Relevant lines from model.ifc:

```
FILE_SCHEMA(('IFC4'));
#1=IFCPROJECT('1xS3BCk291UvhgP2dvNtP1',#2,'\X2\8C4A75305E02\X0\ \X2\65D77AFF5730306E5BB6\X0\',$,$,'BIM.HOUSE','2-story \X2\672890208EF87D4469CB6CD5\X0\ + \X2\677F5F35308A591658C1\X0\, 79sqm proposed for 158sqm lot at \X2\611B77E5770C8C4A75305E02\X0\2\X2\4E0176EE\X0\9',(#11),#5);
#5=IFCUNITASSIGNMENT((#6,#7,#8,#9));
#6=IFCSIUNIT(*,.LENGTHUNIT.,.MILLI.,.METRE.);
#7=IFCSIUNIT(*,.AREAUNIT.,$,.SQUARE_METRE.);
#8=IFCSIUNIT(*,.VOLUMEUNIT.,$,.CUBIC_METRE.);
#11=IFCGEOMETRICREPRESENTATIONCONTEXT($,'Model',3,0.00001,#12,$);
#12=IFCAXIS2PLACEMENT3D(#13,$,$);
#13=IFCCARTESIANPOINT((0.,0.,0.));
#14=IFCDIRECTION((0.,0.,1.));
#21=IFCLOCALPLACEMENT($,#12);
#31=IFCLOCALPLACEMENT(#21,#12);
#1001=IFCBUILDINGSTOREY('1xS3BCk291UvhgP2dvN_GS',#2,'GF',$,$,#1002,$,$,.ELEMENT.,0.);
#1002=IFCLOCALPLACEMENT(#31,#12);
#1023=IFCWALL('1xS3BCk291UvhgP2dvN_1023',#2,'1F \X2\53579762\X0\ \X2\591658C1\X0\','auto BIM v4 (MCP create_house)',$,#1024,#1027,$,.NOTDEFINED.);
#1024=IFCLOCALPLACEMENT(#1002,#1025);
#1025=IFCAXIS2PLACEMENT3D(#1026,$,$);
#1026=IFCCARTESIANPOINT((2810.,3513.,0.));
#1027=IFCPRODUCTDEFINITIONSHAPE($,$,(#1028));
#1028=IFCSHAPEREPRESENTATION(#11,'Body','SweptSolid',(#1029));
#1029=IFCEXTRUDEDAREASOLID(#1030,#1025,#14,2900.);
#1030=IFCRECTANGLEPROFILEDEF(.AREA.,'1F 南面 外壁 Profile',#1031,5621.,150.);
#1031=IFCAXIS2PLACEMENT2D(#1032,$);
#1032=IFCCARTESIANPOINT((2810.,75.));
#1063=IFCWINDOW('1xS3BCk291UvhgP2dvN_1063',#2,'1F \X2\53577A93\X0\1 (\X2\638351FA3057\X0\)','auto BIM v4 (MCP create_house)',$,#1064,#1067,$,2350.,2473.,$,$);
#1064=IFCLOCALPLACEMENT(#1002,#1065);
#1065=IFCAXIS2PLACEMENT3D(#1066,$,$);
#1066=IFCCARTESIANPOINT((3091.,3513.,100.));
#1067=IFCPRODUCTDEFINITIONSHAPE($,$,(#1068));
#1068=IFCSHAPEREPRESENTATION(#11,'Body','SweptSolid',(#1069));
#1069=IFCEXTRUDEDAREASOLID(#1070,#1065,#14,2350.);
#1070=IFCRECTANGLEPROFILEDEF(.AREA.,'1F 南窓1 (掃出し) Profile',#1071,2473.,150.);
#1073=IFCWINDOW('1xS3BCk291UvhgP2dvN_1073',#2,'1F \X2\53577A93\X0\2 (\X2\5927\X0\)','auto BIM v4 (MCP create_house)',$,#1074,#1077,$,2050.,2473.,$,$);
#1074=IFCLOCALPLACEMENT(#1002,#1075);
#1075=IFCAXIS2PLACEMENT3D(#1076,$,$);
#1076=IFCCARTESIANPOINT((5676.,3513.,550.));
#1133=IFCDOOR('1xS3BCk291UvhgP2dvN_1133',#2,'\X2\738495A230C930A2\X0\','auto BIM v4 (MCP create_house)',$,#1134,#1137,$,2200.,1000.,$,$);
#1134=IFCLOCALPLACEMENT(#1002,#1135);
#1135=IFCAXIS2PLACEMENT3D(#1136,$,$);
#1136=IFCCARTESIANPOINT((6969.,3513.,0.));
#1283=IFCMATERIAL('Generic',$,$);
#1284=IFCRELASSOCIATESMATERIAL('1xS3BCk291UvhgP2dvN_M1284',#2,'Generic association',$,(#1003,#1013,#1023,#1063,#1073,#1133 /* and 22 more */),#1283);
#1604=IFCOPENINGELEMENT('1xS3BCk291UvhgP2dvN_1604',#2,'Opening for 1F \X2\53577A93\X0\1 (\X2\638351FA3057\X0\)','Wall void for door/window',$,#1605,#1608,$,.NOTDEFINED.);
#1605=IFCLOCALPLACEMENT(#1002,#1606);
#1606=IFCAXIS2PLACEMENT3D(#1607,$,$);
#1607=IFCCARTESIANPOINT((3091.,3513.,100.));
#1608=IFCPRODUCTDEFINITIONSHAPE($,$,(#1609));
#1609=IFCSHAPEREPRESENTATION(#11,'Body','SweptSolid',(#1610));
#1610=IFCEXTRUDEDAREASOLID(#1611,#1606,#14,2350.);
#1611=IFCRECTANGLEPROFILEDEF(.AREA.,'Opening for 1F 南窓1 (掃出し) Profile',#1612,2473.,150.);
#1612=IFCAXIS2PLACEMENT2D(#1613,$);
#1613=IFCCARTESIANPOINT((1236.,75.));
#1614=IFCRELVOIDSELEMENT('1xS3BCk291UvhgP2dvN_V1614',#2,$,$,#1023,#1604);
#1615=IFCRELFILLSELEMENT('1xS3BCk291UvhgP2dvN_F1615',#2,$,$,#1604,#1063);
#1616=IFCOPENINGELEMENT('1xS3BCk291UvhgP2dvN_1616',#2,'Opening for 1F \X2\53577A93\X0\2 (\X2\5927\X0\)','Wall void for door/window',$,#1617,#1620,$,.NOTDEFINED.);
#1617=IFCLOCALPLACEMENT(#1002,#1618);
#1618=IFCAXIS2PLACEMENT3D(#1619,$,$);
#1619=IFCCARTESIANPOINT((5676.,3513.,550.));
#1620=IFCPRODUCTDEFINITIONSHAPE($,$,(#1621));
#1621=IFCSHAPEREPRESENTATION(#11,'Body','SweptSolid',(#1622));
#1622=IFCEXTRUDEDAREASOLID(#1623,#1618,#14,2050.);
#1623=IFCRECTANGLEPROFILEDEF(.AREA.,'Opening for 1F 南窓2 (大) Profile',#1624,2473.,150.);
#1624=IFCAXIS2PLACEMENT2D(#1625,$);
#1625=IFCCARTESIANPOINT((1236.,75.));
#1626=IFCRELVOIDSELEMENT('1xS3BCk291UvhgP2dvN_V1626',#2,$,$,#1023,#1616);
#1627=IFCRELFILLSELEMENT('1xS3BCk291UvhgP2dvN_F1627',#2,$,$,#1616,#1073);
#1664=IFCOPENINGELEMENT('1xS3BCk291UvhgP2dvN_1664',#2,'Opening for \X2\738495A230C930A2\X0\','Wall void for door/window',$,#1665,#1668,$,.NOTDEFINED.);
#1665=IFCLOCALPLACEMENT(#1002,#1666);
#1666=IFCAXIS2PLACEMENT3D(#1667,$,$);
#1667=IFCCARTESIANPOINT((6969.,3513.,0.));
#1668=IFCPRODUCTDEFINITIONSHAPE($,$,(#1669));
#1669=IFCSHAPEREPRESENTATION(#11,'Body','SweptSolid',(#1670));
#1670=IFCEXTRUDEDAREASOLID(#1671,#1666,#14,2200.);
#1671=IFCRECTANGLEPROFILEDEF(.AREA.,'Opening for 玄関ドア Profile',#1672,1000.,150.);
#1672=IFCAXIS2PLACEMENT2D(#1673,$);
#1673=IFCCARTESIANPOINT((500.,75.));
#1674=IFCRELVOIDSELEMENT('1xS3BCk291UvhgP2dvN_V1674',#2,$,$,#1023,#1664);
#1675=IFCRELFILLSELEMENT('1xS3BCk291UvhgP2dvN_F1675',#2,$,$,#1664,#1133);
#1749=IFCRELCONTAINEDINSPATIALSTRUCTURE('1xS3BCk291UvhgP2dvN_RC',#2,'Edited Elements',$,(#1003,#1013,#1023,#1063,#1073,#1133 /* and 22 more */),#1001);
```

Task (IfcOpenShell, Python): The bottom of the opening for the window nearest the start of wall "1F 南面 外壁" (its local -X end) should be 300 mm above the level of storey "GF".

```python
import numpy as np
import ifcopenshell
import ifcopenshell.api.geometry
import ifcopenshell.geom
import ifcopenshell.util.element
import ifcopenshell.util.placement
import ifcopenshell.util.shape
import ifcopenshell.util.unit

model = ifcopenshell.open("model.ifc")
unit_scale = ifcopenshell.util.unit.calculate_unit_scale(model)

window = model.by_guid("1xS3BCk291UvhgP2dvN_1063")
opening = window.FillsVoids[0].RelatingOpeningElement
storey = ifcopenshell.util.element.get_container(window, ifc_class="IfcBuildingStorey")
level = ifcopenshell.util.placement.get_local_placement(storey.ObjectPlacement)[2, 3]

# The opening's origin need not be at the sill, so measure its lowest point.
shape = ifcopenshell.geom.create_shape(ifcopenshell.geom.settings(), opening)
bottom = ifcopenshell.util.shape.get_shape_bottom_elevation(shape, shape.geometry) / unit_scale
dz = level + 300.0 - bottom

shift = np.array([0.0, 0.0, dz])
# The window is not placed relative to its opening, so move both.
for product in (opening, window):
    matrix = ifcopenshell.util.placement.get_local_placement(product.ObjectPlacement)
    matrix[:3, 3] += shift
    ifcopenshell.api.geometry.edit_object_placement(model, product=product, matrix=matrix, is_si=False)

print(f"moved by {dz * unit_scale:+.3f} m")

model.write("model_rev.ifc")
```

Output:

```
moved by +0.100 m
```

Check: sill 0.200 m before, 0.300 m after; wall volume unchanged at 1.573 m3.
